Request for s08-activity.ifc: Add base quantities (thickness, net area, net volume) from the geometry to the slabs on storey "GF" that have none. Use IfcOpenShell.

First a look at what the model holds.

```python
import ifcopenshell
import ifcopenshell.util.element
import ifcopenshell.util.unit

model = ifcopenshell.open("s08-activity.ifc")
print(model.schema)
for unit_type in ("LENGTHUNIT", "AREAUNIT", "VOLUMEUNIT"):
    print(unit_type, ifcopenshell.util.unit.calculate_unit_scale(model, unit_type))
storey = next(s for s in model.by_type("IfcBuildingStorey") if s.Name == "GF")
slabs = [e for e in ifcopenshell.util.element.get_decomposition(storey) if e.is_a("IfcSlab")]
for e in sorted(slabs, key=lambda e: e.id()):
    print(e.id(), e.is_a(), e.Name, list(ifcopenshell.util.element.get_psets(e, qtos_only=True)), sep=" | ")
```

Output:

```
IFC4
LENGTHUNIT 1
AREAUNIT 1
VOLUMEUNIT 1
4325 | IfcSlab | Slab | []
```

```python
import ifcopenshell
import ifcopenshell.api.pset
import ifcopenshell.geom
import ifcopenshell.util.element
import ifcopenshell.util.shape
import ifcopenshell.util.unit

model = ifcopenshell.open("s08-activity.ifc")
unit_scale = ifcopenshell.util.unit.calculate_unit_scale(model)
area_scale = ifcopenshell.util.unit.calculate_unit_scale(model, "AREAUNIT")
volume_scale = ifcopenshell.util.unit.calculate_unit_scale(model, "VOLUMEUNIT")
settings = ifcopenshell.geom.settings()

storey = next(s for s in model.by_type("IfcBuildingStorey") if s.Name == "GF")
slabs = [e for e in ifcopenshell.util.element.get_decomposition(storey) if e.is_a("IfcSlab")]

for e in sorted(slabs, key=lambda e: e.id()):
    if ifcopenshell.util.element.get_psets(e, qtos_only=True, should_inherit=False):
        continue
    # Geometry comes back in metres, in the element's own axes.
    shape = ifcopenshell.geom.create_shape(settings, e)
    values = {
        "Width": ifcopenshell.util.shape.get_z(shape.geometry) / unit_scale,
        "NetArea": ifcopenshell.util.shape.get_footprint_area(shape.geometry) / area_scale,
        "NetVolume": ifcopenshell.util.shape.get_volume(shape.geometry) / volume_scale,
    }
    qto = ifcopenshell.api.pset.add_qto(model, product=e, name="Qto_SlabBaseQuantities")
    ifcopenshell.api.pset.edit_qto(model, qto=qto, properties=values)
    print(e.id(), {k: round(v, 3) for k, v in values.items()})

model.write("s08-activity_v2.ifc")
```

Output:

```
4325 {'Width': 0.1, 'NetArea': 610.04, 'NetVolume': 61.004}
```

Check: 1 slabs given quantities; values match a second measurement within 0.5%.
